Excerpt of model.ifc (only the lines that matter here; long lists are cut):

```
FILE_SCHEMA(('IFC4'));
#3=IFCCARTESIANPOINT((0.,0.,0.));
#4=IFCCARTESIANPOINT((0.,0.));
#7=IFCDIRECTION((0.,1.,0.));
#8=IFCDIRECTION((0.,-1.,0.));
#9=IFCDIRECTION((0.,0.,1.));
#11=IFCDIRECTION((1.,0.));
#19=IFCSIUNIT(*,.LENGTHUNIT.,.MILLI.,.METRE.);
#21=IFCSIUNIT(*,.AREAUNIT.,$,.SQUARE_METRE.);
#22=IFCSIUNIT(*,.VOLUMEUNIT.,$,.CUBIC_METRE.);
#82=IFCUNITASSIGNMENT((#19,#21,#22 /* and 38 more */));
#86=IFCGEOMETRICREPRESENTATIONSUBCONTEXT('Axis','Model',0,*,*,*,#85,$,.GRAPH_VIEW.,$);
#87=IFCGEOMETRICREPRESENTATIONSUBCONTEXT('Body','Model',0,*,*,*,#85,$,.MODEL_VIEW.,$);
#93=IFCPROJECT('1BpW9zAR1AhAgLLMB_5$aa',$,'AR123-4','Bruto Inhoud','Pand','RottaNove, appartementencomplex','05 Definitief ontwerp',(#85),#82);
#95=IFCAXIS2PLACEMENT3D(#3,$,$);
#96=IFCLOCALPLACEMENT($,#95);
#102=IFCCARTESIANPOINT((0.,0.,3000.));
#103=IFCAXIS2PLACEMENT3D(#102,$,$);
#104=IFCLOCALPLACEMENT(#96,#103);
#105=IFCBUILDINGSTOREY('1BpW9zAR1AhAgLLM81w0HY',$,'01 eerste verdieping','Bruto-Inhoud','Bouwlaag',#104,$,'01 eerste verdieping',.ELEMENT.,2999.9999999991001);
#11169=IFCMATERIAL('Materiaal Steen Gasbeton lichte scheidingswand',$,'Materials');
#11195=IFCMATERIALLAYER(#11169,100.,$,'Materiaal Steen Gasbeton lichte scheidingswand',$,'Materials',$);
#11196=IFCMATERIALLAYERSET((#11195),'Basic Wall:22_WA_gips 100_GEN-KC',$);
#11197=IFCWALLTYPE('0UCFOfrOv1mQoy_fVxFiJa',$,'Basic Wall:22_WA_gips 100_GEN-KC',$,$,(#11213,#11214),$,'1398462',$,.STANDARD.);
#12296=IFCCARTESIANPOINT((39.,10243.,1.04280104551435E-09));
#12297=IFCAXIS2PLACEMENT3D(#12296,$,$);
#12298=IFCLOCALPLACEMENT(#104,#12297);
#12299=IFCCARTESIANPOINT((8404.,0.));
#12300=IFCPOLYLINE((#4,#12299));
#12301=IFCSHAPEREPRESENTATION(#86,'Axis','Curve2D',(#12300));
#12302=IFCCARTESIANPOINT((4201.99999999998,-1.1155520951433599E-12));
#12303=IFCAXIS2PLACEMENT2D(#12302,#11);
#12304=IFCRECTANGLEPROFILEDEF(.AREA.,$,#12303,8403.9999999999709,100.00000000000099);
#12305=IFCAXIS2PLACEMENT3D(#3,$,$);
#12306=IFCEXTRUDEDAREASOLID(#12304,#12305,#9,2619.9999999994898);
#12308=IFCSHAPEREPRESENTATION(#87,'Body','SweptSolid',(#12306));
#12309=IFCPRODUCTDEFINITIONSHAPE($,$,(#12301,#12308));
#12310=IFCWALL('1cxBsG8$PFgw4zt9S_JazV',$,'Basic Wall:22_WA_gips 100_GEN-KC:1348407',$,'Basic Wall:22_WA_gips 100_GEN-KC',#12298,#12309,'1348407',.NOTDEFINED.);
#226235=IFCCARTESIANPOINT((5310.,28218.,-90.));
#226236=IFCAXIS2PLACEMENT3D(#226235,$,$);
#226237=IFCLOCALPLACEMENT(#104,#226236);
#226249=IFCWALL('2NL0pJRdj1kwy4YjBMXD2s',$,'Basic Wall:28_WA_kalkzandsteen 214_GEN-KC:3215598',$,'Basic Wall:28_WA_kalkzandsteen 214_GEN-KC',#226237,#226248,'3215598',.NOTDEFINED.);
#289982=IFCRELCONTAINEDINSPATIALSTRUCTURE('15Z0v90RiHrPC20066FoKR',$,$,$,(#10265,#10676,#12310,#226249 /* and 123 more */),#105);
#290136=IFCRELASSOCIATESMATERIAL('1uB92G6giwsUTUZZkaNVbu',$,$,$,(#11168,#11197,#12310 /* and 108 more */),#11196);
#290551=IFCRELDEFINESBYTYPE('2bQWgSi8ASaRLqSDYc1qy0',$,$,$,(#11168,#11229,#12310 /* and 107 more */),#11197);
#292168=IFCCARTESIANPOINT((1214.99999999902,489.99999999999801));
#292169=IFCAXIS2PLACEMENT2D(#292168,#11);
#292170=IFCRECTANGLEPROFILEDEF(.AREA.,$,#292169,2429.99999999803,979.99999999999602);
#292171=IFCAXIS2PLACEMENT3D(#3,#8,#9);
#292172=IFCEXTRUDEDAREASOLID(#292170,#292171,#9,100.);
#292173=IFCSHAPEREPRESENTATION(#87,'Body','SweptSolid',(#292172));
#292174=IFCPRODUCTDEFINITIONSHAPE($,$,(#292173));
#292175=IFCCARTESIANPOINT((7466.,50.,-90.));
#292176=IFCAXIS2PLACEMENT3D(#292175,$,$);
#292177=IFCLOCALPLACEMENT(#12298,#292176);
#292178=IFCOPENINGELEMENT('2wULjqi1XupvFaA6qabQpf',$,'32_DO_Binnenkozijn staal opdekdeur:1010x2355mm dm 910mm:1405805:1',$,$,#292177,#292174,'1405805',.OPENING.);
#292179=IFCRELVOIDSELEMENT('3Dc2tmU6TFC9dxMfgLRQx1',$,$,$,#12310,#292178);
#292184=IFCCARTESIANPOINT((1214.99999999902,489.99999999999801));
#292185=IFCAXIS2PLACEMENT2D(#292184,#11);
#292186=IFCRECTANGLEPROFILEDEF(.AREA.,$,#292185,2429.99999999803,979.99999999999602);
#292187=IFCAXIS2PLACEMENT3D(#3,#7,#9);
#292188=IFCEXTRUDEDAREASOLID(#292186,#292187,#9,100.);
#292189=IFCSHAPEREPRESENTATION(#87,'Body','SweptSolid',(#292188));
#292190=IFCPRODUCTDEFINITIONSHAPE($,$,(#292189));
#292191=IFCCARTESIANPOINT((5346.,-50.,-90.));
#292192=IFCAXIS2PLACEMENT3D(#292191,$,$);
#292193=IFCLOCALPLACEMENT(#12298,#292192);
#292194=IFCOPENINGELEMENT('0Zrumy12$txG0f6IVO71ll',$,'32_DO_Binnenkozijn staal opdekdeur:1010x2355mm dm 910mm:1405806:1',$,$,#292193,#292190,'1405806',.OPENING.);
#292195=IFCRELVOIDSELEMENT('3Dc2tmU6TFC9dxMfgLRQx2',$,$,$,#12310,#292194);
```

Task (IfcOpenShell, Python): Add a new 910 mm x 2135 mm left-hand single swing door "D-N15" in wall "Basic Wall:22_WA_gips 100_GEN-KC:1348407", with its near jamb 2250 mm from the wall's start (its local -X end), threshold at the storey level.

```python
import numpy as np
import ifcopenshell
import ifcopenshell.api.feature
import ifcopenshell.api.geometry
import ifcopenshell.api.root
import ifcopenshell.api.spatial
import ifcopenshell.geom
import ifcopenshell.util.element
import ifcopenshell.util.placement
import ifcopenshell.util.representation
import ifcopenshell.util.shape
import ifcopenshell.util.unit

model = ifcopenshell.open("model.ifc")
unit_scale = ifcopenshell.util.unit.calculate_unit_scale(model)
settings = ifcopenshell.geom.settings()


def volume(element):
    """Net volume in cubic metres, openings subtracted."""
    shape = ifcopenshell.geom.create_shape(settings, element)
    return ifcopenshell.util.shape.get_volume(shape.geometry)


wall = model.by_id(12310)
storey = ifcopenshell.util.element.get_container(wall, ifc_class="IfcBuildingStorey")
context = ifcopenshell.util.representation.get_context(model, "Model", "Body", "MODEL_VIEW")
before = volume(wall)

width, height, from_end, sill = 0.91, 2.135, 2.25, 0.0  # metres

# The wall runs along its own X axis, and the end named is its -X end.
wall_shape = ifcopenshell.geom.create_shape(settings, wall)
x, y, z = ifcopenshell.util.shape.get_vertices(wall_shape.geometry).T
start = x.min() + from_end
face, thickness = float(y.min()), float(y.max() - y.min())
wall_matrix = ifcopenshell.util.placement.get_local_placement(wall.ObjectPlacement)
level = ifcopenshell.util.placement.get_local_placement(storey.ObjectPlacement)[2, 3]


def in_wall(x, y):
    """Placement at x, y metres in the wall's axes, at sill height."""
    matrix = wall_matrix.copy()
    matrix[:, 3] = wall_matrix @ np.array([x / unit_scale, y / unit_scale, 0.0, 1.0])
    matrix[2, 3] = level + sill / unit_scale
    return matrix


# Opening: a box that overshoots both wall faces by 50 mm.
opening = ifcopenshell.api.root.create_entity(model, ifc_class="IfcOpeningElement", predefined_type="OPENING")
box = ifcopenshell.api.geometry.add_wall_representation(
    model, context=context, length=width, height=height, thickness=thickness + 0.1
)
ifcopenshell.api.geometry.assign_representation(model, product=opening, representation=box)
ifcopenshell.api.geometry.edit_object_placement(model, product=opening, matrix=in_wall(start, face - 0.05), is_si=False)
ifcopenshell.api.feature.add_feature(model, feature=opening, element=wall)

door = ifcopenshell.api.root.create_entity(model, ifc_class="IfcDoor", name="D-N15", predefined_type="DOOR")
door.OverallWidth, door.OverallHeight = width / unit_scale, height / unit_scale
door.OperationType = "SINGLE_SWING_LEFT"
body = ifcopenshell.api.geometry.add_door_representation(
    model,
    context=context,
    overall_width=door.OverallWidth,
    overall_height=door.OverallHeight,
    operation_type="SINGLE_SWING_LEFT",
    lining_properties={"LiningDepth": thickness / unit_scale, "ThresholdDepth": thickness / unit_scale},
)
ifcopenshell.api.geometry.assign_representation(model, product=door, representation=body)
ifcopenshell.api.spatial.assign_container(model, products=[door], relating_structure=storey)
ifcopenshell.api.feature.add_filling(model, opening=opening, element=door)

# The lining spans the wall, so the door starts at the wall face.
ifcopenshell.api.geometry.edit_object_placement(model, product=door, matrix=in_wall(start, face), is_si=False)

after = volume(wall)

print(f"wall volume {before:.3f} -> {after:.3f} m3")

model.write("model_rev.ifc")
```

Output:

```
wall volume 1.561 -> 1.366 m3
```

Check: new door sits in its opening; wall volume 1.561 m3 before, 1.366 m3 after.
